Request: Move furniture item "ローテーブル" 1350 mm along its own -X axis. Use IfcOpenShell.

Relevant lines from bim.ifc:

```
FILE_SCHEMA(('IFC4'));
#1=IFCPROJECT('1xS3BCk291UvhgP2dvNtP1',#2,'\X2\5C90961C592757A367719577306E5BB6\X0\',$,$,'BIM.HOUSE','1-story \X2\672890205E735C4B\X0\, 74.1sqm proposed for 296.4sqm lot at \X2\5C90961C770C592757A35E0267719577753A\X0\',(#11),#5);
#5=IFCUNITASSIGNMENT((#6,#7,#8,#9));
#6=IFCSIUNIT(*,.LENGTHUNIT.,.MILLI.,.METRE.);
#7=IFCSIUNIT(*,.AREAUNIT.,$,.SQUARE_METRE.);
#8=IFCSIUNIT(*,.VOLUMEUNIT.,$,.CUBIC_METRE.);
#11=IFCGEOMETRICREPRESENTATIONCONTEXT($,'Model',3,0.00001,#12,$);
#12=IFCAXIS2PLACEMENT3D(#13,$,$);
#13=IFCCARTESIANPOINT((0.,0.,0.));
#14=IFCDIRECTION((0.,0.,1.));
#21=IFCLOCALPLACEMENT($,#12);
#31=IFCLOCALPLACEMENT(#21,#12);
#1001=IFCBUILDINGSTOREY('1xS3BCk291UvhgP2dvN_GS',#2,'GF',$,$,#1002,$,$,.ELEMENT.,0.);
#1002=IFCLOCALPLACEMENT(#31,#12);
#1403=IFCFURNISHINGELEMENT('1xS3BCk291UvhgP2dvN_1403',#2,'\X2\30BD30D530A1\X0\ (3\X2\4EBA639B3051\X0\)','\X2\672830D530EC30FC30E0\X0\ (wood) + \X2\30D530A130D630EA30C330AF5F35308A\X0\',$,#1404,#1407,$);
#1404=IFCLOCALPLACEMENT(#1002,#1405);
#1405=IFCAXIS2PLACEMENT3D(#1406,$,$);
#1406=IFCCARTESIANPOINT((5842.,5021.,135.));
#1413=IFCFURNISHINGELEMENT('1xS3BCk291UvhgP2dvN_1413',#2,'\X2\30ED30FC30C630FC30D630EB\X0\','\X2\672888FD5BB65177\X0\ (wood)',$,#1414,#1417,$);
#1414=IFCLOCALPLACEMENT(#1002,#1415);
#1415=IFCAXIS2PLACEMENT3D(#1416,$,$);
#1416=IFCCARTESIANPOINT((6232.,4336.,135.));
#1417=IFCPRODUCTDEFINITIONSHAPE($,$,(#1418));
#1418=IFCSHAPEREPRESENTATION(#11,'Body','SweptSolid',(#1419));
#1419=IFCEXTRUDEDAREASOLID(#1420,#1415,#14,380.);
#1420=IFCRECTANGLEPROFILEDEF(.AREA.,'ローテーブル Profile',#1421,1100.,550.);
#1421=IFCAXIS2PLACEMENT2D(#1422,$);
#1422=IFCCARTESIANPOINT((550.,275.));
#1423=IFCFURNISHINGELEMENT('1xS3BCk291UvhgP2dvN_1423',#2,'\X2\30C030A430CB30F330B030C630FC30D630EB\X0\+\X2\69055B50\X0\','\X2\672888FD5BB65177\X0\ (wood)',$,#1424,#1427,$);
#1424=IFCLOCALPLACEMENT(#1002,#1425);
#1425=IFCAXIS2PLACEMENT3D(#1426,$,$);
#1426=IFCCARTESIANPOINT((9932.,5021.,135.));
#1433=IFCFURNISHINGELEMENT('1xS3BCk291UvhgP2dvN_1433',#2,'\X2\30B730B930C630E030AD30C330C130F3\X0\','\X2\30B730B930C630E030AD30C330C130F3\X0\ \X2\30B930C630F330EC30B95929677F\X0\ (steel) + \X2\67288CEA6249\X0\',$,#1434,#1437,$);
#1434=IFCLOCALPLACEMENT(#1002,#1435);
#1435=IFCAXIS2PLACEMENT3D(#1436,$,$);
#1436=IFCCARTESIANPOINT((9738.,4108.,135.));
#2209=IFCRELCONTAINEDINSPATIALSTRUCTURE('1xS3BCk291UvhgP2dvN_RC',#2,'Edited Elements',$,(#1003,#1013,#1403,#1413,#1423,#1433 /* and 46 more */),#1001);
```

```python
import ifcopenshell
import ifcopenshell.api.geometry
import ifcopenshell.util.placement
import ifcopenshell.util.unit

model = ifcopenshell.open("bim.ifc")
unit_scale = ifcopenshell.util.unit.calculate_unit_scale(model)

item = model.by_guid("1xS3BCk291UvhgP2dvN_1413")
matrix = ifcopenshell.util.placement.get_local_placement(item.ObjectPlacement)
matrix[:3, 3] -= matrix[:3, 0] * 1.35 / unit_scale
ifcopenshell.api.geometry.edit_object_placement(model, product=item, matrix=matrix, is_si=False)

print(ifcopenshell.util.placement.get_local_placement(item.ObjectPlacement).round(3) + 0.0)

model.write("bim_v2.ifc")
```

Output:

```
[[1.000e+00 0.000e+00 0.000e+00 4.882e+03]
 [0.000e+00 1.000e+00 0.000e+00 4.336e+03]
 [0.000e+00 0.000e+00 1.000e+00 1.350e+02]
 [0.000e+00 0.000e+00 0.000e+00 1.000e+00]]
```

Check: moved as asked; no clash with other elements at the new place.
